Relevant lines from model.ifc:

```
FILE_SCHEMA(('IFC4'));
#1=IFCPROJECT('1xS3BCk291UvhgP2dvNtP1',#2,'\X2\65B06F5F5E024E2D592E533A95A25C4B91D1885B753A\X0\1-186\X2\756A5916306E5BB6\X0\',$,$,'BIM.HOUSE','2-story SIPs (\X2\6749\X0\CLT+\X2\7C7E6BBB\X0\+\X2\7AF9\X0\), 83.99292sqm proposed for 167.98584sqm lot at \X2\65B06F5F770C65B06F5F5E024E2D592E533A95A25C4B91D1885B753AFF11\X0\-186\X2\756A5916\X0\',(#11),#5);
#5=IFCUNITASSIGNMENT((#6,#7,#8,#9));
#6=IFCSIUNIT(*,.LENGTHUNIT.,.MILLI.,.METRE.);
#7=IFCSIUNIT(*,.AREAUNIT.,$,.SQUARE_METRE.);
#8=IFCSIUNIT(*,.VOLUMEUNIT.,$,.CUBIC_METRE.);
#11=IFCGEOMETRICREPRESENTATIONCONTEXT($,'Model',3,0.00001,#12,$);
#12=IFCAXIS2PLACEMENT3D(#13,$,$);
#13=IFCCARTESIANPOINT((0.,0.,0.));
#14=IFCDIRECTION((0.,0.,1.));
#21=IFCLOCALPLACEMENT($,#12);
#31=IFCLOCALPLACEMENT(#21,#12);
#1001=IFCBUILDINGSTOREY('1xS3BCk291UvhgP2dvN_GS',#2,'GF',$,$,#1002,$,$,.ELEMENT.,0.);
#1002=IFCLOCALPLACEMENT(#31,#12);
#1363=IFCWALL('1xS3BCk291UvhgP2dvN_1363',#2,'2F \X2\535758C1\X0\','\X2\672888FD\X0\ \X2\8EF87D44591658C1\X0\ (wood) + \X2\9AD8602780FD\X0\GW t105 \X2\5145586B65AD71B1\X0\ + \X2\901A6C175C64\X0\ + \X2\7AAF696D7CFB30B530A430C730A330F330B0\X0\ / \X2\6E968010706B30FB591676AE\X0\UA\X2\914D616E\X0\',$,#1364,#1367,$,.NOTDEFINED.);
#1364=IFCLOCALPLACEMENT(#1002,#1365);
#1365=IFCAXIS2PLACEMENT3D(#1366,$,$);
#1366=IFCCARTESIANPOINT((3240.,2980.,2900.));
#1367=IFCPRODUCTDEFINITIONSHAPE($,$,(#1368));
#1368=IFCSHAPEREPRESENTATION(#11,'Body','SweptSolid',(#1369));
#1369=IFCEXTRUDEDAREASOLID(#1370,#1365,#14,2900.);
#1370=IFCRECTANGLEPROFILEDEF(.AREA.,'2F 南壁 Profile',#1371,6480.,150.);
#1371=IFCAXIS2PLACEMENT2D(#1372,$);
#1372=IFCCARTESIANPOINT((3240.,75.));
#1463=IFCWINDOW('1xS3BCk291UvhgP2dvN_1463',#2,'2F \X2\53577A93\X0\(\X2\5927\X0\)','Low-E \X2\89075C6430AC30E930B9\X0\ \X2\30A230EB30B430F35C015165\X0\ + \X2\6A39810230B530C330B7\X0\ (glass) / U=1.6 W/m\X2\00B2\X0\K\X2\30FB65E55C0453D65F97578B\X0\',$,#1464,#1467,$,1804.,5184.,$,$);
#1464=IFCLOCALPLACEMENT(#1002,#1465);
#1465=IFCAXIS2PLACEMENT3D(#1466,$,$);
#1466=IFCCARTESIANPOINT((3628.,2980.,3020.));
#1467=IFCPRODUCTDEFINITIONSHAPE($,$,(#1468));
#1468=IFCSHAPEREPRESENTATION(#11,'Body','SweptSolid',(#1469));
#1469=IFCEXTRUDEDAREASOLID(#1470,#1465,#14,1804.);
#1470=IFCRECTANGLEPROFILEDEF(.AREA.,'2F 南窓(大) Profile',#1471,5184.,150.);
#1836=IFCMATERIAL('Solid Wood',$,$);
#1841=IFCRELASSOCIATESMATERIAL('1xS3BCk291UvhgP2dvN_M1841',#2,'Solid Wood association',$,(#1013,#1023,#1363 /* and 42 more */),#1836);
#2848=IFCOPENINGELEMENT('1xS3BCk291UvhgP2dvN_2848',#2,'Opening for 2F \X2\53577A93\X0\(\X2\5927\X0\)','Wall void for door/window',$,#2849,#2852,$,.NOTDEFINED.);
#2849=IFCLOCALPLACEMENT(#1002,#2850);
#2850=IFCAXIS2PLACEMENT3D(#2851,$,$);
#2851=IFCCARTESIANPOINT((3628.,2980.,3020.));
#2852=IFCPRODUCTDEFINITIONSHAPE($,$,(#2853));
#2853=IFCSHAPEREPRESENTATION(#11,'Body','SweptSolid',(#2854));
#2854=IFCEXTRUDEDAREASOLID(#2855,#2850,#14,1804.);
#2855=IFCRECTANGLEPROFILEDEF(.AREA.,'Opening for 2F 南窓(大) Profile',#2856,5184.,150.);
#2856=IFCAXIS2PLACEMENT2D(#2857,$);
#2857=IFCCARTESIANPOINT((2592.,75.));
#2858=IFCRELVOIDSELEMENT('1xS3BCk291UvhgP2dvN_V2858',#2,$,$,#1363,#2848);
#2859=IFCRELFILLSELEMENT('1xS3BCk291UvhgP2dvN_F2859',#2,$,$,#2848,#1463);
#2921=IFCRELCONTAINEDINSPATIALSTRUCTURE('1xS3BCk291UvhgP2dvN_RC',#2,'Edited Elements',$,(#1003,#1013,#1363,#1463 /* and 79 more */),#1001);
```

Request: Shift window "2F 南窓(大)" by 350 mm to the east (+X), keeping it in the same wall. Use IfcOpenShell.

```python
import ifcopenshell
import ifcopenshell.api.geometry
import ifcopenshell.util.placement
import ifcopenshell.util.unit

model = ifcopenshell.open("model.ifc")
unit_scale = ifcopenshell.util.unit.calculate_unit_scale(model)

window = model.by_guid("1xS3BCk291UvhgP2dvN_1463")
opening = window.FillsVoids[0].RelatingOpeningElement
wall = opening.VoidsElements[0].RelatingBuildingElement

wall_matrix = ifcopenshell.util.placement.get_local_placement(wall.ObjectPlacement)
shift = wall_matrix[:3, 0] * 0.35 / unit_scale
before = ifcopenshell.util.placement.get_local_placement(window.ObjectPlacement)[:3, 3].copy()

# The window is not placed relative to its opening, so move both.
for product in (opening, window):
    matrix = ifcopenshell.util.placement.get_local_placement(product.ObjectPlacement)
    matrix[:3, 3] += shift
    ifcopenshell.api.geometry.edit_object_placement(model, product=product, matrix=matrix, is_si=False)

after = ifcopenshell.util.placement.get_local_placement(window.ObjectPlacement)[:3, 3]
print("window moved by", (after - before).round(3) + 0.0)

model.write("model_edited.ifc")
```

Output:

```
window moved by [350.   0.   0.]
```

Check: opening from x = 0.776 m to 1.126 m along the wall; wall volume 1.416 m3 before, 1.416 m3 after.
